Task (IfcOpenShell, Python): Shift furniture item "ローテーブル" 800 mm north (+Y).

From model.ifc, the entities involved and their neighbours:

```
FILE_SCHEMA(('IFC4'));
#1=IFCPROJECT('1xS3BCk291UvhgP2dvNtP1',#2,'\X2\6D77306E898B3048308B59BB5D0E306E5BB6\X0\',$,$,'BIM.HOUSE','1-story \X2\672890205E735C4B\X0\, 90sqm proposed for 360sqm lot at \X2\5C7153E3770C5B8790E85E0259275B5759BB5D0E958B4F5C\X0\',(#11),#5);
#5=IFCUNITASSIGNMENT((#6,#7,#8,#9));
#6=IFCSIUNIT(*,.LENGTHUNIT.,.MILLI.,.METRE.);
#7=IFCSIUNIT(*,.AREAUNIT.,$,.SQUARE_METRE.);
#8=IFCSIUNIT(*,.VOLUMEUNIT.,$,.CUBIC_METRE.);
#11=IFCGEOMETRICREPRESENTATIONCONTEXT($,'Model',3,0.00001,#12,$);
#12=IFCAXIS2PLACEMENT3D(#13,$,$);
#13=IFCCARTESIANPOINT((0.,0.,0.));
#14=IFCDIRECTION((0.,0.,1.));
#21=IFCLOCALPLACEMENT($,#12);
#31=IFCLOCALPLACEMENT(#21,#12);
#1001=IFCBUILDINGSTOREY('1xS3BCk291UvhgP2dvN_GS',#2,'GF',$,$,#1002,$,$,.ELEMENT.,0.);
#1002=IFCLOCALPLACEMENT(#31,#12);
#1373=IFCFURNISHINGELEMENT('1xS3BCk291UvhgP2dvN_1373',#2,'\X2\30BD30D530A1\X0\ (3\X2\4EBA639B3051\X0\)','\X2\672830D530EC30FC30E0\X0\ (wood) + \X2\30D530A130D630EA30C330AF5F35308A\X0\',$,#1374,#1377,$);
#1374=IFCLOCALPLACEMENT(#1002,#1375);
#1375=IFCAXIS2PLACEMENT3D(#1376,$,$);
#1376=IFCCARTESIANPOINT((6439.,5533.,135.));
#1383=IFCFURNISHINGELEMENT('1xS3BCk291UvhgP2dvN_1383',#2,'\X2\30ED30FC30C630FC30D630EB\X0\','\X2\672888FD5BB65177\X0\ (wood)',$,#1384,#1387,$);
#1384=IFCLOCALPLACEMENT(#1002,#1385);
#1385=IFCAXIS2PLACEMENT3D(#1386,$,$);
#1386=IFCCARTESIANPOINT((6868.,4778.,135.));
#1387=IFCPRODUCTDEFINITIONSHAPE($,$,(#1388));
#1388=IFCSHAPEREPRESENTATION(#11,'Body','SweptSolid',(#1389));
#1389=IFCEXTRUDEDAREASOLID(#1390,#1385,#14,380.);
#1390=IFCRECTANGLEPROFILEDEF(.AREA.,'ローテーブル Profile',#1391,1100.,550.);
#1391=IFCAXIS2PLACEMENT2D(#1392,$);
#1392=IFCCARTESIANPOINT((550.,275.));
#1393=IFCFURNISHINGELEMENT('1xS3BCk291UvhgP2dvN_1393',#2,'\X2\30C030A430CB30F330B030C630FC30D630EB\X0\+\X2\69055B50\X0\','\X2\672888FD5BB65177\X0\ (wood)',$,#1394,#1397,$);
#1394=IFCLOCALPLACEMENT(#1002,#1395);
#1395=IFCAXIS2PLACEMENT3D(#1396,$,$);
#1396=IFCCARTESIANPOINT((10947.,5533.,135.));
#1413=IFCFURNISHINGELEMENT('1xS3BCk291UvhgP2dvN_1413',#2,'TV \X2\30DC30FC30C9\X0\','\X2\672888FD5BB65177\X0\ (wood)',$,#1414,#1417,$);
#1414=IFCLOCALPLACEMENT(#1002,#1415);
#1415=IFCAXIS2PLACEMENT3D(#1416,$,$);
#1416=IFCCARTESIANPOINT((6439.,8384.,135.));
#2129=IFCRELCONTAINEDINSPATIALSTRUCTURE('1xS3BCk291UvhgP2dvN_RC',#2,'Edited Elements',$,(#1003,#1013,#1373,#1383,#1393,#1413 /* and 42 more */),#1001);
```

```python
import ifcopenshell
import ifcopenshell.api.geometry
import ifcopenshell.util.placement

model = ifcopenshell.open("model.ifc")

item = model.by_guid("1xS3BCk291UvhgP2dvN_1383")
matrix = ifcopenshell.util.placement.get_local_placement(item.ObjectPlacement)
matrix[1, 3] += 800.0
ifcopenshell.api.geometry.edit_object_placement(model, product=item, matrix=matrix, is_si=False)

print(ifcopenshell.util.placement.get_local_placement(item.ObjectPlacement).round(3) + 0.0)

model.write("model-out.ifc")
```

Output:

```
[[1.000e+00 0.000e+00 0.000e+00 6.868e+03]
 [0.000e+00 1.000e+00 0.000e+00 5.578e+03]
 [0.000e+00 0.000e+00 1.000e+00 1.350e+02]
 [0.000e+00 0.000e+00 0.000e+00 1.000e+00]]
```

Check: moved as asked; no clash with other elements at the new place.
